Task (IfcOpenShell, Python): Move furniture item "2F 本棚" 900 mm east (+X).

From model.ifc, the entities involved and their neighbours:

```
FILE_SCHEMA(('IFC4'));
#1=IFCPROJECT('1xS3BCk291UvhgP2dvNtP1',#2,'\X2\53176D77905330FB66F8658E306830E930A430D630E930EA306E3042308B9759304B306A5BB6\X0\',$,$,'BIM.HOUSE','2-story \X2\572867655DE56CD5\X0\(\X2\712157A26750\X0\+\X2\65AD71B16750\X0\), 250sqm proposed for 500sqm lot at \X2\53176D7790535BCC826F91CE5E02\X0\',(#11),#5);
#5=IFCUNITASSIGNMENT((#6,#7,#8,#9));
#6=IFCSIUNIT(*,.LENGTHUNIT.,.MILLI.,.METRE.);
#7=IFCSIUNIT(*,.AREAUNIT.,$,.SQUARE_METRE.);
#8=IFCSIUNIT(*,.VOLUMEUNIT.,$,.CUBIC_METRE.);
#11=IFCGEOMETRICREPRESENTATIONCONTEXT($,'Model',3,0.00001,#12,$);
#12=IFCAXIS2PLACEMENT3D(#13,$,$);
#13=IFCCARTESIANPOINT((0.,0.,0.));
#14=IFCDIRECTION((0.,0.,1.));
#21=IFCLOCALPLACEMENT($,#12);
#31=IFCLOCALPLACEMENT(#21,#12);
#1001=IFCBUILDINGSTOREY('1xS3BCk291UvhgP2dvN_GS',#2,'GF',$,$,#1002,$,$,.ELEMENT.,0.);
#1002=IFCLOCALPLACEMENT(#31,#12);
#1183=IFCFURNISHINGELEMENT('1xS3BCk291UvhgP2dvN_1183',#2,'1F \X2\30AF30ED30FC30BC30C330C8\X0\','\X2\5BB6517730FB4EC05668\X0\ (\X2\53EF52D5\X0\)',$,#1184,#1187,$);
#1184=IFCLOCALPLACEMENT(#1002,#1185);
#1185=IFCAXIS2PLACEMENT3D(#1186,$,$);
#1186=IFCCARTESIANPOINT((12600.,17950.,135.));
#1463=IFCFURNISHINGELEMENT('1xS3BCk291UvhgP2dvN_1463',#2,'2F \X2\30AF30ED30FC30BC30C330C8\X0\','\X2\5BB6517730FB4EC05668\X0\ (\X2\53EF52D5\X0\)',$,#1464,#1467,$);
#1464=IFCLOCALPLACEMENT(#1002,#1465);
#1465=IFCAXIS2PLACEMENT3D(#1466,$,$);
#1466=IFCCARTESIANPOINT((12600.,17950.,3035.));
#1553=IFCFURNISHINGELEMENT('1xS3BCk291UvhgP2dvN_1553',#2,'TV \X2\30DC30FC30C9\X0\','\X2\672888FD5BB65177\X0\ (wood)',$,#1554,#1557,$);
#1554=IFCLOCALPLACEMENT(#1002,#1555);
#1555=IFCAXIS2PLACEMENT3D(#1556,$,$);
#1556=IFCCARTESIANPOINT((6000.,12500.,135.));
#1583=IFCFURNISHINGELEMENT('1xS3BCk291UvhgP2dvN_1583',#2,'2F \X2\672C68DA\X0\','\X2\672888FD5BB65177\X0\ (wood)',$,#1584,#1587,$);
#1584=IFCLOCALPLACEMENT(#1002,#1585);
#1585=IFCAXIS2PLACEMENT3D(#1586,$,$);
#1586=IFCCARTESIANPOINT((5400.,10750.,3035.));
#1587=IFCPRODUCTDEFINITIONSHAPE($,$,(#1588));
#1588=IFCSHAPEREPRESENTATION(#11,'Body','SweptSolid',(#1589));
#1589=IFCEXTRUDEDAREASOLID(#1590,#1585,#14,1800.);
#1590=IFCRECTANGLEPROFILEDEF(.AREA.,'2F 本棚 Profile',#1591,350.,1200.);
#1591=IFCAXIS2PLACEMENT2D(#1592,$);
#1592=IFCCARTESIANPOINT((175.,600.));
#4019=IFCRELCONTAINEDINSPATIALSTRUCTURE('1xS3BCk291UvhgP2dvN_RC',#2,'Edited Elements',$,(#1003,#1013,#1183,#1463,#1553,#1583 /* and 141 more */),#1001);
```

```python
import ifcopenshell
import ifcopenshell.api.geometry
import ifcopenshell.util.placement
import ifcopenshell.util.unit

model = ifcopenshell.open("model.ifc")
unit_scale = ifcopenshell.util.unit.calculate_unit_scale(model)

item = model.by_guid("1xS3BCk291UvhgP2dvN_1583")
matrix = ifcopenshell.util.placement.get_local_placement(item.ObjectPlacement)
matrix[0, 3] += 0.9 / unit_scale
ifcopenshell.api.geometry.edit_object_placement(model, product=item, matrix=matrix, is_si=False)

print(ifcopenshell.util.placement.get_local_placement(item.ObjectPlacement).round(3) + 0.0)

model.write("model_updated.ifc")
```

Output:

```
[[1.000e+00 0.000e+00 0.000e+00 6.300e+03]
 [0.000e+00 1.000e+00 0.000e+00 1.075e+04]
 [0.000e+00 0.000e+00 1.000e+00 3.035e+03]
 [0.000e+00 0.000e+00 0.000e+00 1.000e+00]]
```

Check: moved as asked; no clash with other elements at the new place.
